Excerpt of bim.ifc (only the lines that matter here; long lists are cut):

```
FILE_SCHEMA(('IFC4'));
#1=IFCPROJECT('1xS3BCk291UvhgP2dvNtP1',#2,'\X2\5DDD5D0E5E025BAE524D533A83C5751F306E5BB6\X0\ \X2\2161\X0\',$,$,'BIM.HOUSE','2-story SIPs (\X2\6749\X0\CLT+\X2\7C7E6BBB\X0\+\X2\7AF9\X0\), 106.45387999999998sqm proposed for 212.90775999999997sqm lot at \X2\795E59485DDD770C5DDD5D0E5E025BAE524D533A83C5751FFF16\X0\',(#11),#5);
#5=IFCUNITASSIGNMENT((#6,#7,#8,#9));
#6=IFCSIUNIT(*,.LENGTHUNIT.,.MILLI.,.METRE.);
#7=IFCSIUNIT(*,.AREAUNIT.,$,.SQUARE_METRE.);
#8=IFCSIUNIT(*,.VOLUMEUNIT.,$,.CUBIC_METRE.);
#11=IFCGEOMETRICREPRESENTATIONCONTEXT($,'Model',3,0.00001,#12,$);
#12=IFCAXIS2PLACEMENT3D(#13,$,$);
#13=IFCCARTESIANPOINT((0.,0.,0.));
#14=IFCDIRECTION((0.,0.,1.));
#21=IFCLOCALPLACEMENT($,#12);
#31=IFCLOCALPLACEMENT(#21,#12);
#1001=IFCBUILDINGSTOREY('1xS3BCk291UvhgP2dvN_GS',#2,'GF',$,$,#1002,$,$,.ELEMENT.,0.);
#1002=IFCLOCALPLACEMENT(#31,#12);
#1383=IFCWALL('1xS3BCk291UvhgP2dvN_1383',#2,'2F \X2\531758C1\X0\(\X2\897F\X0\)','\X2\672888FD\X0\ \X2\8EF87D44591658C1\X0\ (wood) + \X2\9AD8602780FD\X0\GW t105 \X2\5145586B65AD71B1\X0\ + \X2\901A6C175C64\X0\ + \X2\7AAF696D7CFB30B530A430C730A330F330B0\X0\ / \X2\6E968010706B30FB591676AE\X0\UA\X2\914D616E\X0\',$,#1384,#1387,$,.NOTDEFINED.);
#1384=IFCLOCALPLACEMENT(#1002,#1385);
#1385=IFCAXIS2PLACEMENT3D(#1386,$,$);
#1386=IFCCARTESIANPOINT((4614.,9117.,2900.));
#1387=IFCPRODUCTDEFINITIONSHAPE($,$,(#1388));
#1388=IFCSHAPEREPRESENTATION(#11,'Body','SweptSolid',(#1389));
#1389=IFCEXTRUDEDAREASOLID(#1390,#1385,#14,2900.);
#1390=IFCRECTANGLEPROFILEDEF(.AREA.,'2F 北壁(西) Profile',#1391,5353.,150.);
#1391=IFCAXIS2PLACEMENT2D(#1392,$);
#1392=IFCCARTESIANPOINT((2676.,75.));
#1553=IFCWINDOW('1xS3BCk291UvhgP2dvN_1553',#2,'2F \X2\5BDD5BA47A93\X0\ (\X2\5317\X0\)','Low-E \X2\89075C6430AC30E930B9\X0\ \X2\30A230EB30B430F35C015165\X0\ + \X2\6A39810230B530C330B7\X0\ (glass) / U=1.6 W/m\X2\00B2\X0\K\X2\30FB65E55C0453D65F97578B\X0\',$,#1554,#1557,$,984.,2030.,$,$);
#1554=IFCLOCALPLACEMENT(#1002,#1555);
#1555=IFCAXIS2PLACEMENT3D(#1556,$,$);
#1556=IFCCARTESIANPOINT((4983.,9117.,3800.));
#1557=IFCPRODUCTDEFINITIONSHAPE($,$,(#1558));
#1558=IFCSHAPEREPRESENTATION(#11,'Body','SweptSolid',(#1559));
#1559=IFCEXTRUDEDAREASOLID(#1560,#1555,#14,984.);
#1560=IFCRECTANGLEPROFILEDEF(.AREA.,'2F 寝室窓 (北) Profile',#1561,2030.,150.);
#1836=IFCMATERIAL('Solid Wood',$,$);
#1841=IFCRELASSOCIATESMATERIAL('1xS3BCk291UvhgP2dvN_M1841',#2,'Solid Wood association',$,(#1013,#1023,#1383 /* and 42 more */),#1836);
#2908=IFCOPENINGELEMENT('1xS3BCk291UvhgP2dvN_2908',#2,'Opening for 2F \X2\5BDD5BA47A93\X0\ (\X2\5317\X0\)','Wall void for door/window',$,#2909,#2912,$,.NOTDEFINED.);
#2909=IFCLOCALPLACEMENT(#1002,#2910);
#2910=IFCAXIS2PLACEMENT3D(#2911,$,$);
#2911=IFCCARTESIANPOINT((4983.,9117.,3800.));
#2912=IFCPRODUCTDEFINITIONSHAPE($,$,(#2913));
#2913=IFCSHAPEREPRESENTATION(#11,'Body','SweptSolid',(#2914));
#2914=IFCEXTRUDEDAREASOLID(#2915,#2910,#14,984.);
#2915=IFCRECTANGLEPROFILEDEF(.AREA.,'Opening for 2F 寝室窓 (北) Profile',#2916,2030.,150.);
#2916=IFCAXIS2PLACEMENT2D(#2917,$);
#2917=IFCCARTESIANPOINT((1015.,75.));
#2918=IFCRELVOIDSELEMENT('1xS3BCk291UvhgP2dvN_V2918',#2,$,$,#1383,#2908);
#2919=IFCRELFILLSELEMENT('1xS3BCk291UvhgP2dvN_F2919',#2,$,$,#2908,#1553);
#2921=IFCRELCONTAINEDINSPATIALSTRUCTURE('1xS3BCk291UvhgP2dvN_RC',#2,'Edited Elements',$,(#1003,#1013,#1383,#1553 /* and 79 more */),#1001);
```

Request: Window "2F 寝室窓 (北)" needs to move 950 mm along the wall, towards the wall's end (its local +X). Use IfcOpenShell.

```python
import ifcopenshell
import ifcopenshell.api.geometry
import ifcopenshell.util.placement
import ifcopenshell.util.unit

model = ifcopenshell.open("bim.ifc")
unit_scale = ifcopenshell.util.unit.calculate_unit_scale(model)

window = model.by_guid("1xS3BCk291UvhgP2dvN_1553")
opening = window.FillsVoids[0].RelatingOpeningElement
wall = opening.VoidsElements[0].RelatingBuildingElement

wall_matrix = ifcopenshell.util.placement.get_local_placement(wall.ObjectPlacement)
shift = wall_matrix[:3, 0] * 0.95 / unit_scale
before = ifcopenshell.util.placement.get_local_placement(window.ObjectPlacement)[:3, 3].copy()

# The window is not placed relative to its opening, so move both.
for product in (opening, window):
    matrix = ifcopenshell.util.placement.get_local_placement(product.ObjectPlacement)
    matrix[:3, 3] += shift
    ifcopenshell.api.geometry.edit_object_placement(model, product=product, matrix=matrix, is_si=False)

after = ifcopenshell.util.placement.get_local_placement(window.ObjectPlacement)[:3, 3]
print("window moved by", (after - before).round(3) + 0.0)

model.write("bim-out.ifc")
```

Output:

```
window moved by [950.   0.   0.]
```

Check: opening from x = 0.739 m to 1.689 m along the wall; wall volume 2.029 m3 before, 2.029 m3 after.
